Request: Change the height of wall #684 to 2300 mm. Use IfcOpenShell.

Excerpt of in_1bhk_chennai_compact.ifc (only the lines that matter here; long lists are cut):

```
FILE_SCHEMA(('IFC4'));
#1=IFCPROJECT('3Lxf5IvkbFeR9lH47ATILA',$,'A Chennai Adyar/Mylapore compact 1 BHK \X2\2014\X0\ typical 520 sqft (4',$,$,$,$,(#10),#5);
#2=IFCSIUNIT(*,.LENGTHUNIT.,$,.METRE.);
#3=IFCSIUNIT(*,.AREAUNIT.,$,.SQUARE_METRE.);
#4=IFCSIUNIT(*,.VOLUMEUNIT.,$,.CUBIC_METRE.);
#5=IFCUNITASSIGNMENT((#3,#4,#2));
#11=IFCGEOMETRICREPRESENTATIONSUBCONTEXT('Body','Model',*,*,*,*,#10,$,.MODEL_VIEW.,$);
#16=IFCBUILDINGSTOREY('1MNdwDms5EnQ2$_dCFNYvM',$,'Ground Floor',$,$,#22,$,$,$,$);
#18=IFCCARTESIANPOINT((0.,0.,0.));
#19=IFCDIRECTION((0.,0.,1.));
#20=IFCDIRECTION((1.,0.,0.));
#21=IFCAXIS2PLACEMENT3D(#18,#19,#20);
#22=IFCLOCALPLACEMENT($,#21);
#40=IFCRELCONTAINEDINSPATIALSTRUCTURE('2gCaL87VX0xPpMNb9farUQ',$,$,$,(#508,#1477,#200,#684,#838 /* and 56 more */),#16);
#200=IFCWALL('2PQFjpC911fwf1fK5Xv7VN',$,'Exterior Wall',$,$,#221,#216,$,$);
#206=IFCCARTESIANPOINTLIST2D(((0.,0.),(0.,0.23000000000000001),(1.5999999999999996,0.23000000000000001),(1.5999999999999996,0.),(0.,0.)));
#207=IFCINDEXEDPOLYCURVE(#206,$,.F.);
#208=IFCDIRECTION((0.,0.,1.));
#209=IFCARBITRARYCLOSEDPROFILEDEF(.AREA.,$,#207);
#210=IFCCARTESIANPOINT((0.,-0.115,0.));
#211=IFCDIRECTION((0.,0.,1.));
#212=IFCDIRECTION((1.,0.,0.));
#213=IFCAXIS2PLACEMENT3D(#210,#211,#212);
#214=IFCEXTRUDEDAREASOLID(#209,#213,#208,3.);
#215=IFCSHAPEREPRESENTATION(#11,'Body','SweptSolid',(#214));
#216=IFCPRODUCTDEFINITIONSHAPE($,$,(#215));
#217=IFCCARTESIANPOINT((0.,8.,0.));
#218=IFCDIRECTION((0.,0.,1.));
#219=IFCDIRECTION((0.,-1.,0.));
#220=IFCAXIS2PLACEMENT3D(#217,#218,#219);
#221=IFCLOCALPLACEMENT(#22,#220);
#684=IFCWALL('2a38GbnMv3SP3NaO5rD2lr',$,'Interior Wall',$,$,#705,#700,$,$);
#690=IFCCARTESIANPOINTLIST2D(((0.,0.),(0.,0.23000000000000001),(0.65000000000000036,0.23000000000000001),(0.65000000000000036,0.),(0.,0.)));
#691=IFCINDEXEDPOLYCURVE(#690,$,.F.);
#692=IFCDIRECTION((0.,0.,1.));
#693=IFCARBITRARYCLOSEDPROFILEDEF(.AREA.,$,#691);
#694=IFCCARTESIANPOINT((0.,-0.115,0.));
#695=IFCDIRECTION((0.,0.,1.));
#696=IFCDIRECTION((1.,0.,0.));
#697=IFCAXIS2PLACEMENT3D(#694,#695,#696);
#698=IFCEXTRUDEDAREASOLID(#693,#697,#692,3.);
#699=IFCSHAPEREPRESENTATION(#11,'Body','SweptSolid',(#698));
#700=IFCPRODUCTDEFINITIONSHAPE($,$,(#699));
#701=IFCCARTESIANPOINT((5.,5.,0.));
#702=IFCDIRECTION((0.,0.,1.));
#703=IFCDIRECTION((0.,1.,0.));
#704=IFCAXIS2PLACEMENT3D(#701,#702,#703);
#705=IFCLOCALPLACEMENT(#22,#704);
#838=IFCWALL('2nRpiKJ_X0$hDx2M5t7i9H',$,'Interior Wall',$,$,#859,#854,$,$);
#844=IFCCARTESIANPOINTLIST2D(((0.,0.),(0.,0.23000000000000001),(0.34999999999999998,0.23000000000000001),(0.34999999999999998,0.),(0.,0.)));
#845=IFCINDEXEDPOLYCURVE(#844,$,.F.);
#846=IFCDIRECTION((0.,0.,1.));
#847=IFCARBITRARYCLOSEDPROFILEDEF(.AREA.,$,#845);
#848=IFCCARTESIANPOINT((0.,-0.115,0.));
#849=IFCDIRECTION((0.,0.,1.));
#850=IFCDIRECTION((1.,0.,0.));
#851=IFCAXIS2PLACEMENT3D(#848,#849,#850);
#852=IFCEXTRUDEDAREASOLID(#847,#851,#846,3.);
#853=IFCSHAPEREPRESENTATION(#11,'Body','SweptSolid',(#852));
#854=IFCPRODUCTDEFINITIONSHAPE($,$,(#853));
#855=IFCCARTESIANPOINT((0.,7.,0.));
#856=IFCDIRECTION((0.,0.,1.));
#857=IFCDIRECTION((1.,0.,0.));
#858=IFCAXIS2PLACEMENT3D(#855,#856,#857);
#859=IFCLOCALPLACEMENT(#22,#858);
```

```python
import ifcopenshell
import ifcopenshell.geom
import ifcopenshell.util.representation
import ifcopenshell.util.shape
import ifcopenshell.util.unit

model = ifcopenshell.open("in_1bhk_chennai_compact.ifc")
unit_scale = ifcopenshell.util.unit.calculate_unit_scale(model)
settings = ifcopenshell.geom.settings()


def volume(element):
    """Net volume in cubic metres, openings subtracted."""
    shape = ifcopenshell.geom.create_shape(settings, element)
    return ifcopenshell.util.shape.get_volume(shape.geometry)


wall = model.by_id(684)
before = volume(wall)

body = ifcopenshell.util.representation.get_representation(wall, "Model", "Body")
solid = body.Items[0]
old_height = solid.Depth
solid.Depth = 2.3 / unit_scale
after = volume(wall)

print(f"height {old_height:g} -> {solid.Depth:g}, volume {before:.3f} -> {after:.3f} m3")

model.write("in_1bhk_chennai_compact_updated.ifc")
```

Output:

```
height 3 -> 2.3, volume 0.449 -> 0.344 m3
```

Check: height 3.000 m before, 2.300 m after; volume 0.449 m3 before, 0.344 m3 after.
